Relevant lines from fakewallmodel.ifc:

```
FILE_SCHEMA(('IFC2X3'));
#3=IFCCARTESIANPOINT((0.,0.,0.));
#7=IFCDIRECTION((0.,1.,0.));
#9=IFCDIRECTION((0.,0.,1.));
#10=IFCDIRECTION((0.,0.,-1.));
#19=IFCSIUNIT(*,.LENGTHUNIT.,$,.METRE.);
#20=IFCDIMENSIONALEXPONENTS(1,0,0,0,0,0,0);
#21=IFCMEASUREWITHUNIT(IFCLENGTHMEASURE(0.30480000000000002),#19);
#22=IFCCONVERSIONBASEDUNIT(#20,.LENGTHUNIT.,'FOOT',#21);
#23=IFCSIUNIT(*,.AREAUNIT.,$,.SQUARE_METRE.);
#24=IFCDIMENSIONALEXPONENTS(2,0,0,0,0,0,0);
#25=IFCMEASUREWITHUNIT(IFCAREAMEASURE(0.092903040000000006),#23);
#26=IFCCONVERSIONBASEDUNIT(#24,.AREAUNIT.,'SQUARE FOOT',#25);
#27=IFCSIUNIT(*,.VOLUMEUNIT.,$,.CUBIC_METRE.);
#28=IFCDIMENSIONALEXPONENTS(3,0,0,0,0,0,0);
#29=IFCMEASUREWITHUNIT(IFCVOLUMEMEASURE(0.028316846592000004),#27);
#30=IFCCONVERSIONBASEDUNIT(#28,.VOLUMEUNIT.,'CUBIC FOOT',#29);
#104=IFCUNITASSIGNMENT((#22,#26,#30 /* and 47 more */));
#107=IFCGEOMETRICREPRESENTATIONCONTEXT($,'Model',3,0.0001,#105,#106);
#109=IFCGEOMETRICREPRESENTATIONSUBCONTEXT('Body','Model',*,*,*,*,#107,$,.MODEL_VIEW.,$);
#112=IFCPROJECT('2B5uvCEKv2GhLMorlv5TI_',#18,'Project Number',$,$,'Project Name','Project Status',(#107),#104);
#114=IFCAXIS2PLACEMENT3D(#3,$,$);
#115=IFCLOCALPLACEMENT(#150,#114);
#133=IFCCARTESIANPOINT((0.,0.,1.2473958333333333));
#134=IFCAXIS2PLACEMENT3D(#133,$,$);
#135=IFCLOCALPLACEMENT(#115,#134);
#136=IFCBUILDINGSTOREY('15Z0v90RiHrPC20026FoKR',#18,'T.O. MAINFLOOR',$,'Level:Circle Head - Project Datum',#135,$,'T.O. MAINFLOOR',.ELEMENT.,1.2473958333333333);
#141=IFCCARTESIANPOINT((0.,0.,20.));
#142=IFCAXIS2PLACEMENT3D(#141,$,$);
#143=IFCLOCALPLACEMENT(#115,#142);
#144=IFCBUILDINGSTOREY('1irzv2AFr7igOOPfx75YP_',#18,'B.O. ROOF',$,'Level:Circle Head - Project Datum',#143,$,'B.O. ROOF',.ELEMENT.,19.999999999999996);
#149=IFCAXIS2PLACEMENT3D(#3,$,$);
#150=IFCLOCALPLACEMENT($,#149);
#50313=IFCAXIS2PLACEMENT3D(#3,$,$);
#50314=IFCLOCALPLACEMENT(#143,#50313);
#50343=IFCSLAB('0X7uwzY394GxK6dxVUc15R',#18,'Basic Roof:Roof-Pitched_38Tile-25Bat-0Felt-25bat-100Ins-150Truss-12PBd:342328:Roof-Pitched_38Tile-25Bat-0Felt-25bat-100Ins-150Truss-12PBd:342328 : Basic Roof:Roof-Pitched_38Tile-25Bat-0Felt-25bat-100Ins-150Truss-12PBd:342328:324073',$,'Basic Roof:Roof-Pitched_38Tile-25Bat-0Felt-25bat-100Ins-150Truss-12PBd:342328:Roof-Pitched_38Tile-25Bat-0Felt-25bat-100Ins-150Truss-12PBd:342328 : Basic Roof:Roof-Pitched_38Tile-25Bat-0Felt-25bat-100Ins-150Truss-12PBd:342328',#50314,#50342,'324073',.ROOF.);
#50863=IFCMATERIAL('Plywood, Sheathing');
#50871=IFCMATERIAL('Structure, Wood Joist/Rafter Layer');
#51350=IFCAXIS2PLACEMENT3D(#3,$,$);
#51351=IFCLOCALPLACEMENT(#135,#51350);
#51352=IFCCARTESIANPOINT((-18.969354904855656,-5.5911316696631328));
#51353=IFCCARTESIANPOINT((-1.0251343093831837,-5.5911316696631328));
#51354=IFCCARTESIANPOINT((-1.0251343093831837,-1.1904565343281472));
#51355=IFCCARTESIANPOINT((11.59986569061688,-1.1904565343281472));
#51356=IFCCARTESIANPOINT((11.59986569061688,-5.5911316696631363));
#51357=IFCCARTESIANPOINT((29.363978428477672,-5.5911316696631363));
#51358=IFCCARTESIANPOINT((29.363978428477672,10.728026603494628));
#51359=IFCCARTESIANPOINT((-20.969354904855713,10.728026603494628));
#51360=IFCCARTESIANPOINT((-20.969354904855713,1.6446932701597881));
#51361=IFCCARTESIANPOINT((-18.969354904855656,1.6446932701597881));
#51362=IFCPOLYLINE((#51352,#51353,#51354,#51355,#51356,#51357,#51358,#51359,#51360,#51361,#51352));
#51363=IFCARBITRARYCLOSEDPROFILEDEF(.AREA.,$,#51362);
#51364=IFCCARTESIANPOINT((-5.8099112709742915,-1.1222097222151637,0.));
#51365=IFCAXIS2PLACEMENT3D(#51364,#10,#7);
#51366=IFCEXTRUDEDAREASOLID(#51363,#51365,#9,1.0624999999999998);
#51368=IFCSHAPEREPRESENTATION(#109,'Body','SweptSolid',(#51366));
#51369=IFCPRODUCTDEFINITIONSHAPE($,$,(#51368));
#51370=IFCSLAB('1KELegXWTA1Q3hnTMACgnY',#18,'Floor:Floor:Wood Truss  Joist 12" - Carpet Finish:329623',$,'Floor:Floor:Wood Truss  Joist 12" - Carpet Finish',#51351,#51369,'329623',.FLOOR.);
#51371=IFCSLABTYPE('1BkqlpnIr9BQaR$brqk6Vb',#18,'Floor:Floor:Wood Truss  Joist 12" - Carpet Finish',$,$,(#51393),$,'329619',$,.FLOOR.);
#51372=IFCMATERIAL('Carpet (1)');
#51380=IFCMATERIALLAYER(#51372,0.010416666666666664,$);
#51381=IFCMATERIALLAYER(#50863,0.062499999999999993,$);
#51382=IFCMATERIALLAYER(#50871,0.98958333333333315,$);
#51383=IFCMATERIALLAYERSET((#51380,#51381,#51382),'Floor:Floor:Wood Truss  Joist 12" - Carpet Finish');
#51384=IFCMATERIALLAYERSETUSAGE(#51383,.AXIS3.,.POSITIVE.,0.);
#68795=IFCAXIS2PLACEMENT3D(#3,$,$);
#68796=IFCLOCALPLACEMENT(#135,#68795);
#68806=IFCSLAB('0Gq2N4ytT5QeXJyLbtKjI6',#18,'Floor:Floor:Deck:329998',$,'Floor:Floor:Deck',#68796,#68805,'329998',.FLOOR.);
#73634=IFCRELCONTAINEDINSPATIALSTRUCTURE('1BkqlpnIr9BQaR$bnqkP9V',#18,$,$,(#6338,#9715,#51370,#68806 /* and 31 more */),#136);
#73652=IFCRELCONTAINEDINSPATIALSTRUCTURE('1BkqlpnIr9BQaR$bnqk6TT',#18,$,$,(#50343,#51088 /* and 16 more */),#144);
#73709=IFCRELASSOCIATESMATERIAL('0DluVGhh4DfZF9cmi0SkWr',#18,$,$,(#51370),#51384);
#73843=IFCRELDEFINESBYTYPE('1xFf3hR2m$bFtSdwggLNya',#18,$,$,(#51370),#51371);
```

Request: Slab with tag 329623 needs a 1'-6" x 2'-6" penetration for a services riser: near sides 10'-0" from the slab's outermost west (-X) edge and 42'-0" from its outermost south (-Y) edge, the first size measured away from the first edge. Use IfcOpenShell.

```python
import numpy as np
import ifcopenshell
import ifcopenshell.api.feature
import ifcopenshell.api.geometry
import ifcopenshell.api.root
import ifcopenshell.geom
import ifcopenshell.util.placement
import ifcopenshell.util.representation
import ifcopenshell.util.shape
import ifcopenshell.util.unit

model = ifcopenshell.open("fakewallmodel.ifc")
unit_scale = ifcopenshell.util.unit.calculate_unit_scale(model)
settings = ifcopenshell.geom.settings()


def volume(element):
    """Net volume in cubic metres, openings subtracted."""
    shape = ifcopenshell.geom.create_shape(settings, element)
    return ifcopenshell.util.shape.get_volume(shape.geometry)


slab = model.by_id(51370)
before = volume(slab)

# Extent in the slab's own axes, in metres. The edges named are its -X and -Y sides.
slab_shape = ifcopenshell.geom.create_shape(settings, slab)
vertices = ifcopenshell.util.shape.get_vertices(slab_shape.geometry)
x_min, y_min, bottom = vertices.min(axis=0)
top = vertices[:, 2].max()

opening = ifcopenshell.api.root.create_entity(model, ifc_class="IfcOpeningElement", name="Services riser opening")
context = ifcopenshell.util.representation.get_context(model, "Model", "Body", "MODEL_VIEW")
width, depth = 0.4572, 0.762
outline = [(0.0, 0.0), (width, 0.0), (width, depth), (0.0, depth), (0.0, 0.0)]
# Overshoot both faces by 50 mm so the cut is clean.
shape = ifcopenshell.api.geometry.add_slab_representation(
    model, context=context, depth=top - bottom + 0.1, polyline=outline
)
ifcopenshell.api.geometry.assign_representation(model, product=opening, representation=shape)

matrix = ifcopenshell.util.placement.get_local_placement(slab.ObjectPlacement)
matrix[:, 3] = matrix @ np.append(np.array([x_min + 3.048, y_min + 12.8016, bottom - 0.05]) / unit_scale, 1.0)
ifcopenshell.api.geometry.edit_object_placement(model, product=opening, matrix=matrix, is_si=False)
ifcopenshell.api.feature.add_feature(model, feature=opening, element=slab)

after = volume(slab)

print(f"slab volume {before:.3f} -> {after:.3f} m3")

model.write("fakewallmodel_rev.ifc")
```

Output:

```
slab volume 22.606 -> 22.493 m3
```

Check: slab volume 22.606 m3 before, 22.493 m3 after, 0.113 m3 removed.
